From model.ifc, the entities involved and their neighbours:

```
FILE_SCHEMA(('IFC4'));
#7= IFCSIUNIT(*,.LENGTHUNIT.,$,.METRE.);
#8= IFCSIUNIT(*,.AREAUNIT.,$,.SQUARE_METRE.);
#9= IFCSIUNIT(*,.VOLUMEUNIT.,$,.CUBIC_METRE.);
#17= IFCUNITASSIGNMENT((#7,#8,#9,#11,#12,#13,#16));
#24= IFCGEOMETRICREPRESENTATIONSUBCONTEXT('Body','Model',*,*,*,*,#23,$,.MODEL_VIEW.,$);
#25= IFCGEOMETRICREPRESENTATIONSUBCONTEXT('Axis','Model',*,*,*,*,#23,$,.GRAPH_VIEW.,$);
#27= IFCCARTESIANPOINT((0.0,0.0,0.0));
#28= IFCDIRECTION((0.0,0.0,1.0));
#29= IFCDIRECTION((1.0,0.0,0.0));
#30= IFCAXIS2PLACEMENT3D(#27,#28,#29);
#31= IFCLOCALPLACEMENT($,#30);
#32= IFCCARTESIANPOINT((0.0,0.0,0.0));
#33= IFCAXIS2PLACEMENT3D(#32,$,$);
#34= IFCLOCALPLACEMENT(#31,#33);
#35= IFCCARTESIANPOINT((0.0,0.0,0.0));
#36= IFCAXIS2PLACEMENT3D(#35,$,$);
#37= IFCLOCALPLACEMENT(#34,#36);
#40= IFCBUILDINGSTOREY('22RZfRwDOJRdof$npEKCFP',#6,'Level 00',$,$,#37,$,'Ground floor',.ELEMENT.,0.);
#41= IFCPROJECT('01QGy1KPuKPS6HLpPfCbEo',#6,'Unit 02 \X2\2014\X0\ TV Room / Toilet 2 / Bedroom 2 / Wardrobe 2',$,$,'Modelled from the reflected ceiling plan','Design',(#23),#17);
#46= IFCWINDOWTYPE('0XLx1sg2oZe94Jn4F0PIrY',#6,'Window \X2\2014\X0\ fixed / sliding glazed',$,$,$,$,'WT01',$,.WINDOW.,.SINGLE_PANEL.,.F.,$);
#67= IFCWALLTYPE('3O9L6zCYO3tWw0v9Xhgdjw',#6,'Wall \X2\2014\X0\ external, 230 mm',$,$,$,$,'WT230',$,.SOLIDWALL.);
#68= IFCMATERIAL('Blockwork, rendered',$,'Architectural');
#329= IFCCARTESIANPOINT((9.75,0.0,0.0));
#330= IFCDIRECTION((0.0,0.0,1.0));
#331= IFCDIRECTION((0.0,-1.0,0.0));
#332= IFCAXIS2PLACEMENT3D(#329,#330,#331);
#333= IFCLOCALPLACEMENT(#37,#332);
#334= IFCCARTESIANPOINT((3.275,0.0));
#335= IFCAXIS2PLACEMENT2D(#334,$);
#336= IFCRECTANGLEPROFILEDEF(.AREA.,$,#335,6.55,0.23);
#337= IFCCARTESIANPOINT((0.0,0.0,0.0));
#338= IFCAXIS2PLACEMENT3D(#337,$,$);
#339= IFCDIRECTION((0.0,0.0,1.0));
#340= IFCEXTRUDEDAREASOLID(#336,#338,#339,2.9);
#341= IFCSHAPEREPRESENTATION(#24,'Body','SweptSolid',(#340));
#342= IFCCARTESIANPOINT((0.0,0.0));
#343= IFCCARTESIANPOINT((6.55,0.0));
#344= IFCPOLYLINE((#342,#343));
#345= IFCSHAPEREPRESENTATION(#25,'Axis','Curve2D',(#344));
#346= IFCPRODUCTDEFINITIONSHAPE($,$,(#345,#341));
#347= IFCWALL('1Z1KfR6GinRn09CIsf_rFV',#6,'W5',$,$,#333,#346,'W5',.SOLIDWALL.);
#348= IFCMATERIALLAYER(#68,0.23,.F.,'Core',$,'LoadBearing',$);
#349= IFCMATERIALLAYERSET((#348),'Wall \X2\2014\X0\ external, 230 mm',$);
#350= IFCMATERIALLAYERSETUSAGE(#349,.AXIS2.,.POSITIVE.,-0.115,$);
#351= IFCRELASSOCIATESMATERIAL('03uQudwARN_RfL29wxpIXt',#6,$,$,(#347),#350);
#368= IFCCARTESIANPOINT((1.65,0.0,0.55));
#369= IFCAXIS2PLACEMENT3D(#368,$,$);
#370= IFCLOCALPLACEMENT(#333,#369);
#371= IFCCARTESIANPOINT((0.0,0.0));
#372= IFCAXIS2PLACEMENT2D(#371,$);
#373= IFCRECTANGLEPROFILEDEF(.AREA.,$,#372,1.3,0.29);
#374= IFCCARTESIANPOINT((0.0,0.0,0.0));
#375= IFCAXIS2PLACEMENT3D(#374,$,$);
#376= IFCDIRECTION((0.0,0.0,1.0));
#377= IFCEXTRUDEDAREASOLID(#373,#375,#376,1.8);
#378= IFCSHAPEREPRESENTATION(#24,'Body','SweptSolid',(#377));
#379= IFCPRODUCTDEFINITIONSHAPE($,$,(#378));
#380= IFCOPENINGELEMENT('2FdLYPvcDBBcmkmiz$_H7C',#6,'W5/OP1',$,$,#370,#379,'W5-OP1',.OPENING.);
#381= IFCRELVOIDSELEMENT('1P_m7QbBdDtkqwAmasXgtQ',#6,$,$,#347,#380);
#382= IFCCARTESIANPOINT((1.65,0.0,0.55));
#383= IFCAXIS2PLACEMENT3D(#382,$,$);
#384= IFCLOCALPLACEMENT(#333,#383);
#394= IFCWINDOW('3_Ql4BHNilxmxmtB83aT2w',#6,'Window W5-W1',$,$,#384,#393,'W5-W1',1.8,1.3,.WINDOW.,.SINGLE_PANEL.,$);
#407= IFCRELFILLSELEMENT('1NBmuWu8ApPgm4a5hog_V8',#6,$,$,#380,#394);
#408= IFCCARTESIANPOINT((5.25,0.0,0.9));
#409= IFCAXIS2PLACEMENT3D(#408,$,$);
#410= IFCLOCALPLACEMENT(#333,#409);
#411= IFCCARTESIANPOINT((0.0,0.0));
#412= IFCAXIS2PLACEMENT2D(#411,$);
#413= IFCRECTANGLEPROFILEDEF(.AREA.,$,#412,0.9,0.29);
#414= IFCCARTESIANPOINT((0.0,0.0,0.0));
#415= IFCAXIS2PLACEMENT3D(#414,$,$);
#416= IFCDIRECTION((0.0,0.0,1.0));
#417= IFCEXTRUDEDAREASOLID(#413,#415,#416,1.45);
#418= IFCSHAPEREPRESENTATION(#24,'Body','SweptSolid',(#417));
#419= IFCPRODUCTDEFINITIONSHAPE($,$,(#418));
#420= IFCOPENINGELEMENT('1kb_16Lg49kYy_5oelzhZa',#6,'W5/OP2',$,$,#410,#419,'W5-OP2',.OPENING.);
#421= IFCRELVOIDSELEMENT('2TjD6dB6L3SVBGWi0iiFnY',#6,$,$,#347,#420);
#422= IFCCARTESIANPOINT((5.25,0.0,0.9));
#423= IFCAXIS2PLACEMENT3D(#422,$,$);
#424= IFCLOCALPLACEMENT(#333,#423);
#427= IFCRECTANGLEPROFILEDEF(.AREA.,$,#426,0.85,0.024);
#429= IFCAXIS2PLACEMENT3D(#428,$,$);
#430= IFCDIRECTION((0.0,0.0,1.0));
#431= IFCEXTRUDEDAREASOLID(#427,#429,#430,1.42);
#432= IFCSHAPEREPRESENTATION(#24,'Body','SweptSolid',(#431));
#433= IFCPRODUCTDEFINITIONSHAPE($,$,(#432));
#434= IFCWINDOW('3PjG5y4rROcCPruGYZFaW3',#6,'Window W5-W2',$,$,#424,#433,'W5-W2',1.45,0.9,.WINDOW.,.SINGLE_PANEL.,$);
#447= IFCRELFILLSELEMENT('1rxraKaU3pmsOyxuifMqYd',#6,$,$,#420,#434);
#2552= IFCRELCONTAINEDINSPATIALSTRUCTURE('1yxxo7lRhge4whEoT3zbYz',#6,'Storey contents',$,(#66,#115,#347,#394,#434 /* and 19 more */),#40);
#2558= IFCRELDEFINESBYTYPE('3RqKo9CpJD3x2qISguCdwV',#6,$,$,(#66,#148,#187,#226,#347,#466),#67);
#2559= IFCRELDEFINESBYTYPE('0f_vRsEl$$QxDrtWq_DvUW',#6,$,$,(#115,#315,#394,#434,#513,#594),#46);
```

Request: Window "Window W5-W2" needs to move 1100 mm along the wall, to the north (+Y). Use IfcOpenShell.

```python
import ifcopenshell
import ifcopenshell.api.geometry
import ifcopenshell.util.placement
import ifcopenshell.util.unit

model = ifcopenshell.open("model.ifc")
unit_scale = ifcopenshell.util.unit.calculate_unit_scale(model)

window = model.by_id(434)
opening = window.FillsVoids[0].RelatingOpeningElement
wall = opening.VoidsElements[0].RelatingBuildingElement

wall_matrix = ifcopenshell.util.placement.get_local_placement(wall.ObjectPlacement)
shift = wall_matrix[:3, 0] * -1.1 / unit_scale
before = ifcopenshell.util.placement.get_local_placement(window.ObjectPlacement)[:3, 3].copy()

# The window is not placed relative to its opening, so move both.
for product in (opening, window):
    matrix = ifcopenshell.util.placement.get_local_placement(product.ObjectPlacement)
    matrix[:3, 3] += shift
    ifcopenshell.api.geometry.edit_object_placement(model, product=product, matrix=matrix, is_si=False)

after = ifcopenshell.util.placement.get_local_placement(window.ObjectPlacement)[:3, 3]
print("window moved by", (after - before).round(3) + 0.0)

model.write("model-out.ifc")
```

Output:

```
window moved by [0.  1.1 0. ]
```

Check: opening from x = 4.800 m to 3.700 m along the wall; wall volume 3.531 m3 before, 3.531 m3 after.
